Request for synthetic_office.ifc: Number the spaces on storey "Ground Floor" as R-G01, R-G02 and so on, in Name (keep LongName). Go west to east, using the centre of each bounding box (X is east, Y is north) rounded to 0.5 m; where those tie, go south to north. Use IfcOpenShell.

First a look at what the model holds.

```python
import ifcopenshell
import ifcopenshell.util.element
import ifcopenshell.util.placement

model = ifcopenshell.open("synthetic_office.ifc")
print(model.schema)
storey = next(s for s in model.by_type("IfcBuildingStorey") if s.Name == "Ground Floor")
spaces = [e for e in ifcopenshell.util.element.get_decomposition(storey) if e.is_a("IfcSpace")]
for e in sorted(spaces, key=lambda e: e.id()):
    origin = ifcopenshell.util.placement.get_local_placement(e.ObjectPlacement)[:3, 3]
    print(e.id(), e.Name, e.LongName, origin.round(2) + 0.0, sep=" | ")
```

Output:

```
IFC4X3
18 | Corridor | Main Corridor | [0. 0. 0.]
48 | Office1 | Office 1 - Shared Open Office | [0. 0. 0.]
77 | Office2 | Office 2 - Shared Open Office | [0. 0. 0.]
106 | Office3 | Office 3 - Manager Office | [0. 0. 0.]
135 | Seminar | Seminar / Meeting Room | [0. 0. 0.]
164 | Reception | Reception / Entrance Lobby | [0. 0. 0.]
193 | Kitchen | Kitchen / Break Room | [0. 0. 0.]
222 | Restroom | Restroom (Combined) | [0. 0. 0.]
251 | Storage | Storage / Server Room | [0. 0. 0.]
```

```python
import ifcopenshell
import ifcopenshell.geom
import ifcopenshell.util.element
import ifcopenshell.util.shape

model = ifcopenshell.open("synthetic_office.ifc")
settings = ifcopenshell.geom.settings()
settings.set("use-world-coords", True)


def centre(element):
    shape = ifcopenshell.geom.create_shape(settings, element)
    return ifcopenshell.util.shape.get_bbox_centroid(shape.geometry)


storey = next(s for s in model.by_type("IfcBuildingStorey") if s.Name == "Ground Floor")
spaces = [e for e in ifcopenshell.util.element.get_decomposition(storey) if e.is_a("IfcSpace")]

# Insertion points can sit at a corner or the storey origin, so sort by the geometry (in metres).
centres = {e: centre(e) for e in spaces}
spaces.sort(key=lambda e: (round(centres[e][0] / 0.5), centres[e][1]))

for i, e in enumerate(spaces, start=1):
    number = f"R-G{i:02d}"
    e.Name = number
    print(e.id(), number)

model.write("synthetic_office_edited.ifc")
```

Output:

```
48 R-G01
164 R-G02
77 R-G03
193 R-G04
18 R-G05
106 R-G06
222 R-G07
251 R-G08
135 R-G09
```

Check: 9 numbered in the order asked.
